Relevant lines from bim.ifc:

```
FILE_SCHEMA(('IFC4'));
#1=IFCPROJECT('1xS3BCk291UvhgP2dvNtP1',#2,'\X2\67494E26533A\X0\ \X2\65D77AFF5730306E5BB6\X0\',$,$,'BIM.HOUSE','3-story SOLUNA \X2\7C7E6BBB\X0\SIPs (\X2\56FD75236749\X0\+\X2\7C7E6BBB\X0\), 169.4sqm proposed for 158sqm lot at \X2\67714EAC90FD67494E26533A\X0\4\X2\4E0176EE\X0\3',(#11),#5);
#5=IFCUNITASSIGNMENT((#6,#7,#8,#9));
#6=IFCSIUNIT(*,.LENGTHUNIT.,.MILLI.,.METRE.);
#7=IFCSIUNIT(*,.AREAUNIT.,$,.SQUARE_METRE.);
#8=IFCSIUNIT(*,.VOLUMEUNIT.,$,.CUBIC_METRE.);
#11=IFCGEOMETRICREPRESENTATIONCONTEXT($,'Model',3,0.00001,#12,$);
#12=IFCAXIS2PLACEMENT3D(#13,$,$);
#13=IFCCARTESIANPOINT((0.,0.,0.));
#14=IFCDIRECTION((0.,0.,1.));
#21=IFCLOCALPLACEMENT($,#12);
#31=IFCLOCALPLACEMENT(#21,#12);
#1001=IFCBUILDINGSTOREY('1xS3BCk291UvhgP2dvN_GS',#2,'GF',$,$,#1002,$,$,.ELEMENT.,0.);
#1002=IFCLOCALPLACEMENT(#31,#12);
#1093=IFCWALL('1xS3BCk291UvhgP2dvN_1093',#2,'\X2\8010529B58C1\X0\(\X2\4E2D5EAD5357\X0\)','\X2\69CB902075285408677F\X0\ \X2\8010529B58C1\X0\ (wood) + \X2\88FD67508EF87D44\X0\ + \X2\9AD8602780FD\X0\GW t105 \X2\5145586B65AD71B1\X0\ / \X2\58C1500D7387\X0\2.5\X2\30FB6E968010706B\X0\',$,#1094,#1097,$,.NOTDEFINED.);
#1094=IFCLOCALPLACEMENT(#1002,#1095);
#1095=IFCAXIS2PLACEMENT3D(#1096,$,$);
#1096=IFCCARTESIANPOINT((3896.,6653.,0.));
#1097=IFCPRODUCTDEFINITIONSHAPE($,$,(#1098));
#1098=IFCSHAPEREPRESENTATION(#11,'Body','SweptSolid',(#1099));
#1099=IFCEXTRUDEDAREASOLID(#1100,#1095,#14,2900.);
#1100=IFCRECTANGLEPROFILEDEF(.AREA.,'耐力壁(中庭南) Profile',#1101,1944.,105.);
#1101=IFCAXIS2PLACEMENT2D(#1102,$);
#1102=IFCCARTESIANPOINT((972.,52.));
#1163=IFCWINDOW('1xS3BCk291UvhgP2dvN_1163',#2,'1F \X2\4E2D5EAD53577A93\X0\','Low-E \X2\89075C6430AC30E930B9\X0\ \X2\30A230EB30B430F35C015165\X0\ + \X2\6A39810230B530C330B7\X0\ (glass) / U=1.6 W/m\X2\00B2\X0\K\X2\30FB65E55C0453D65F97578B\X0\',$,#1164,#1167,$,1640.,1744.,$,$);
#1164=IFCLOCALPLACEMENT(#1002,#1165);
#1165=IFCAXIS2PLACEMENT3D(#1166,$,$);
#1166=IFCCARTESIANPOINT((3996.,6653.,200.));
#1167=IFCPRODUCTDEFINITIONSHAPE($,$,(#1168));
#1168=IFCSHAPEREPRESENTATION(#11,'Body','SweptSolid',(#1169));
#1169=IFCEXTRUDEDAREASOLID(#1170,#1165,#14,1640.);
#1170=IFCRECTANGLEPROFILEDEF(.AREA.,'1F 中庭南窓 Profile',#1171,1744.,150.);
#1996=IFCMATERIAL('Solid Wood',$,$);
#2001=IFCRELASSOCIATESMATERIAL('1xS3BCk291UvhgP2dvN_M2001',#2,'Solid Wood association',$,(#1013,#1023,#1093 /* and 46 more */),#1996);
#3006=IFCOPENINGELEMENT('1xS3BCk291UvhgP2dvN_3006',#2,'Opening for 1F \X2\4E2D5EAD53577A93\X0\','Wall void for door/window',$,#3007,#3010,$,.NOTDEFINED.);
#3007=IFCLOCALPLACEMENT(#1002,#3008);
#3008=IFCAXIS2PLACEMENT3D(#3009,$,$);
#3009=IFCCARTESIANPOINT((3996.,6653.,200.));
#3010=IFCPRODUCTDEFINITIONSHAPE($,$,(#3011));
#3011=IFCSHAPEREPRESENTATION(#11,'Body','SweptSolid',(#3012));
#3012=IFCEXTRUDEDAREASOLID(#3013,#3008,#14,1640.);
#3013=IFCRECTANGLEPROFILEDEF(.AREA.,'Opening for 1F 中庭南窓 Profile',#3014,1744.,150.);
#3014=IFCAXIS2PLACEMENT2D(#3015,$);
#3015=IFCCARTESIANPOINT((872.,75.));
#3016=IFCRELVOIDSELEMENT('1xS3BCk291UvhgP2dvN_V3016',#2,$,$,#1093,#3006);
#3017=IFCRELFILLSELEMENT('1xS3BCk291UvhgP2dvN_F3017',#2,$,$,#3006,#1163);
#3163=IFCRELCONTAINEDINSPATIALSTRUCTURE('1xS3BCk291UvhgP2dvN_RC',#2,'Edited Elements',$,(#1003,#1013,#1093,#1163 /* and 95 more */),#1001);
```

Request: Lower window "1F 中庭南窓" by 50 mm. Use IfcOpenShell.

```python
import numpy as np
import ifcopenshell
import ifcopenshell.api.geometry
import ifcopenshell.util.placement
import ifcopenshell.util.unit

model = ifcopenshell.open("bim.ifc")
unit_scale = ifcopenshell.util.unit.calculate_unit_scale(model)

window = model.by_guid("1xS3BCk291UvhgP2dvN_1163")
opening = window.FillsVoids[0].RelatingOpeningElement
dz = -50.0

shift = np.array([0.0, 0.0, dz])
# The window is not placed relative to its opening, so move both.
for product in (opening, window):
    matrix = ifcopenshell.util.placement.get_local_placement(product.ObjectPlacement)
    matrix[:3, 3] += shift
    ifcopenshell.api.geometry.edit_object_placement(model, product=product, matrix=matrix, is_si=False)

print(f"moved by {dz * unit_scale:+.3f} m")

model.write("bim_updated.ifc")
```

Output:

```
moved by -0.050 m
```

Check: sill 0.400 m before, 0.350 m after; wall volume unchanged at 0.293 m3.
